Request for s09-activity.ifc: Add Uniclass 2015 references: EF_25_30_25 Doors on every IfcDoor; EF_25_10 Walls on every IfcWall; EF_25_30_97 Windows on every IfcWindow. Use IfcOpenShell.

First a look at what the model holds.

```python
import ifcopenshell

model = ifcopenshell.open("s09-activity.ifc")
print(model.schema)
print("classifications:", [c.Name for c in model.by_type("IfcClassification")])
for ifc_class in ("IfcDoor", "IfcRoof", "IfcStair", "IfcWall", "IfcWindow"):
    print(ifc_class, len(model.by_type(ifc_class)))
```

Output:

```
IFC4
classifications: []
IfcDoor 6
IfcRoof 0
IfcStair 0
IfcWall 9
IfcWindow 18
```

```python
import ifcopenshell
import ifcopenshell.api.classification

model = ifcopenshell.open("s09-activity.ifc")

system = ifcopenshell.api.classification.add_classification(model, classification="Uniclass 2015")

codes = {
    "IfcDoor": ("EF_25_30_25", "Doors"),
    "IfcWall": ("EF_25_10", "Walls"),
    "IfcWindow": ("EF_25_30_97", "Windows"),
}
for ifc_class, (code, name) in codes.items():
    products = model.by_type(ifc_class)
    ifcopenshell.api.classification.add_reference(
        model, products=products, classification=system, identification=code, name=name
    )
    print(code, len(products))

model.write("s09-activity_rev.ifc")
```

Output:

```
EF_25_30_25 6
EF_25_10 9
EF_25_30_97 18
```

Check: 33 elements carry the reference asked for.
